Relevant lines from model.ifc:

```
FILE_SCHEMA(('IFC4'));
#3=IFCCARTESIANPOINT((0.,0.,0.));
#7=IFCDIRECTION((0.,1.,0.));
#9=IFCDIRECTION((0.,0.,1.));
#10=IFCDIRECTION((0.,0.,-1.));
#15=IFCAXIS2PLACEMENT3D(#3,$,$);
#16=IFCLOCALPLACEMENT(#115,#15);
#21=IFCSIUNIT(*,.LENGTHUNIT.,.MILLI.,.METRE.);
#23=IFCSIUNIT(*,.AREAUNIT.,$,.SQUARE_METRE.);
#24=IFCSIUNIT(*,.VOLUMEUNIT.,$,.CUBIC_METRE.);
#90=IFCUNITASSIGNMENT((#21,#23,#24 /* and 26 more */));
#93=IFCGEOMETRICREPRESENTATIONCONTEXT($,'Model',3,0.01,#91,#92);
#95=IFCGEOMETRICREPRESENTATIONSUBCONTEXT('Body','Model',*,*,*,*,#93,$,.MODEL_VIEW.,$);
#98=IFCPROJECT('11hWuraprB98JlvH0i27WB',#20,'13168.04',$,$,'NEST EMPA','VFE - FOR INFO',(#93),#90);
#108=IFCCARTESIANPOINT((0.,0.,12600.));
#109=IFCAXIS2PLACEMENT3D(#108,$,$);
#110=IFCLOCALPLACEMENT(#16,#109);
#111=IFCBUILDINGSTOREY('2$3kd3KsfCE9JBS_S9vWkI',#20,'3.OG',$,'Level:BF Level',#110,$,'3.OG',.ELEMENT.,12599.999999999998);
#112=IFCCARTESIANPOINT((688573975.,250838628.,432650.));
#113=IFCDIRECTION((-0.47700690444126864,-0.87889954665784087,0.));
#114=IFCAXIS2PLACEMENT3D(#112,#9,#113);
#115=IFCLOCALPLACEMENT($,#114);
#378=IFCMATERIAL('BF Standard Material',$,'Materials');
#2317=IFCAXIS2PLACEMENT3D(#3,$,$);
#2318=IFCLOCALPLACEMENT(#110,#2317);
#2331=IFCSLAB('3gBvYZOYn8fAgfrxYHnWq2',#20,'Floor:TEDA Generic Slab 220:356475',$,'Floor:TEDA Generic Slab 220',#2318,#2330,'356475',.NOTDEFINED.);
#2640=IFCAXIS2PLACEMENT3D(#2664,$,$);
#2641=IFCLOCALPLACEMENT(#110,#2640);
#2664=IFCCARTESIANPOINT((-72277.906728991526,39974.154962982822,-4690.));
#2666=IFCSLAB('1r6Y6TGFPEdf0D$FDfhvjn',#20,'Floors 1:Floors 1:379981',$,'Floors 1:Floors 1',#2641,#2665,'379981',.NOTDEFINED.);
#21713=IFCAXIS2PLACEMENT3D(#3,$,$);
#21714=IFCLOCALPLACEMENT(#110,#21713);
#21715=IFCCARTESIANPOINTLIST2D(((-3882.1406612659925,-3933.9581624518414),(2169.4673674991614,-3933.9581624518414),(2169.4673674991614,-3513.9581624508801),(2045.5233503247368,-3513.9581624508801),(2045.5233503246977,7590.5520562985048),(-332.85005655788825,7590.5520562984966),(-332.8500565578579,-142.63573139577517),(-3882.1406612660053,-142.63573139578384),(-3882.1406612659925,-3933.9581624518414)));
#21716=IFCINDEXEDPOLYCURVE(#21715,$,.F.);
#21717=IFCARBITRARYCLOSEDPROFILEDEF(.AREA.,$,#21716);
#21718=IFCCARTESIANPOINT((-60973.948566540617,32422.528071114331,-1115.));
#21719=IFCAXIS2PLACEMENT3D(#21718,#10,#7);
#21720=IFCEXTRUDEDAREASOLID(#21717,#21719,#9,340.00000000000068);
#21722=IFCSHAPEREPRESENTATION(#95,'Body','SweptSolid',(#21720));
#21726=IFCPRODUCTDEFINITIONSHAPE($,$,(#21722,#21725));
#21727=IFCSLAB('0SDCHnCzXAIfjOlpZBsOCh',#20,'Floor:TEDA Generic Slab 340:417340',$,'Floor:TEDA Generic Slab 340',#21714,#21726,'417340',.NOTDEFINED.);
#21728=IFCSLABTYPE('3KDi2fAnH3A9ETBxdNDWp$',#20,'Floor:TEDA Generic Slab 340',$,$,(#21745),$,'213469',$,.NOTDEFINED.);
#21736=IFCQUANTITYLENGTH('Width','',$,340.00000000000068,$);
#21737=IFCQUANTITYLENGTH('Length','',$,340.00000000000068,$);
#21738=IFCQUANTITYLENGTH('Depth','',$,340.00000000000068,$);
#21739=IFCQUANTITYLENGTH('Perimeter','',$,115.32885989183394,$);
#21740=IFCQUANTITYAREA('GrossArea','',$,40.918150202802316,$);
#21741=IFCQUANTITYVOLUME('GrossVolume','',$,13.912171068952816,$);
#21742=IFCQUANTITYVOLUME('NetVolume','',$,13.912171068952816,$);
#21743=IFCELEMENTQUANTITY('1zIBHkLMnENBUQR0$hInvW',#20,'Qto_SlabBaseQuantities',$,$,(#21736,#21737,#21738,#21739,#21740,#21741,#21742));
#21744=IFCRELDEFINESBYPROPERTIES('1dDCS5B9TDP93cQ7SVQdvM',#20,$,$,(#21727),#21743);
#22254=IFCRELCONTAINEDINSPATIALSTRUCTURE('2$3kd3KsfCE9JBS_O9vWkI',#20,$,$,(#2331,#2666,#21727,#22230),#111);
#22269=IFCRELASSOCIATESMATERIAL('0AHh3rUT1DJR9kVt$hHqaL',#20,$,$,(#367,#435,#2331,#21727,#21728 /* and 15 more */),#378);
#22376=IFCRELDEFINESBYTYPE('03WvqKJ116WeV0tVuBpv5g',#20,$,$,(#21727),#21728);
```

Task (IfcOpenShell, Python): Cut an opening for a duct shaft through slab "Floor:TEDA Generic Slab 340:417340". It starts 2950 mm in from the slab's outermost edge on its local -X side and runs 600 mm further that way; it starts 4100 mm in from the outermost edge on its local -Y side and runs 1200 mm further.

```python
import numpy as np
import ifcopenshell
import ifcopenshell.api.feature
import ifcopenshell.api.geometry
import ifcopenshell.api.pset
import ifcopenshell.api.root
import ifcopenshell.geom
import ifcopenshell.util.element
import ifcopenshell.util.placement
import ifcopenshell.util.representation
import ifcopenshell.util.shape
import ifcopenshell.util.unit

model = ifcopenshell.open("model.ifc")
unit_scale = ifcopenshell.util.unit.calculate_unit_scale(model)
volume_scale = ifcopenshell.util.unit.calculate_unit_scale(model, "VOLUMEUNIT")
settings = ifcopenshell.geom.settings()


def volume(element):
    """Net volume in cubic metres, openings subtracted."""
    shape = ifcopenshell.geom.create_shape(settings, element)
    return ifcopenshell.util.shape.get_volume(shape.geometry)


slab = model.by_id(21727)
before = volume(slab)

# Extent in the slab's own axes, in metres. The edges named are its -X and -Y sides.
slab_shape = ifcopenshell.geom.create_shape(settings, slab)
vertices = ifcopenshell.util.shape.get_vertices(slab_shape.geometry)
x_min, y_min, bottom = vertices.min(axis=0)
top = vertices[:, 2].max()

opening = ifcopenshell.api.root.create_entity(model, ifc_class="IfcOpeningElement", name="Duct shaft opening", predefined_type="OPENING")
context = ifcopenshell.util.representation.get_context(model, "Model", "Body", "MODEL_VIEW")
width, depth = 0.6, 1.2
outline = [(0.0, 0.0), (width, 0.0), (width, depth), (0.0, depth), (0.0, 0.0)]
# Overshoot both faces by 50 mm so the cut is clean.
shape = ifcopenshell.api.geometry.add_slab_representation(
    model, context=context, depth=top - bottom + 0.1, polyline=outline
)
ifcopenshell.api.geometry.assign_representation(model, product=opening, representation=shape)

matrix = ifcopenshell.util.placement.get_local_placement(slab.ObjectPlacement)
matrix[:, 3] = matrix @ np.append(np.array([x_min + 2.95, y_min + 4.1, bottom - 0.05]) / unit_scale, 1.0)
ifcopenshell.api.geometry.edit_object_placement(model, product=opening, matrix=matrix, is_si=False)
ifcopenshell.api.feature.add_feature(model, feature=opening, element=slab)

after = volume(slab)

# Update the slab's stored quantities.
qto = model.by_id(ifcopenshell.util.element.get_pset(slab, "Qto_SlabBaseQuantities", should_inherit=False)["id"])
ifcopenshell.api.pset.edit_qto(model, qto=qto, properties={"NetVolume": after / volume_scale})

print(f"slab volume {before:.3f} -> {after:.3f} m3")

model.write("model-out.ifc")
```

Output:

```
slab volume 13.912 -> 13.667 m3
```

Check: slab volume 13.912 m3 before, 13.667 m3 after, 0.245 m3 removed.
